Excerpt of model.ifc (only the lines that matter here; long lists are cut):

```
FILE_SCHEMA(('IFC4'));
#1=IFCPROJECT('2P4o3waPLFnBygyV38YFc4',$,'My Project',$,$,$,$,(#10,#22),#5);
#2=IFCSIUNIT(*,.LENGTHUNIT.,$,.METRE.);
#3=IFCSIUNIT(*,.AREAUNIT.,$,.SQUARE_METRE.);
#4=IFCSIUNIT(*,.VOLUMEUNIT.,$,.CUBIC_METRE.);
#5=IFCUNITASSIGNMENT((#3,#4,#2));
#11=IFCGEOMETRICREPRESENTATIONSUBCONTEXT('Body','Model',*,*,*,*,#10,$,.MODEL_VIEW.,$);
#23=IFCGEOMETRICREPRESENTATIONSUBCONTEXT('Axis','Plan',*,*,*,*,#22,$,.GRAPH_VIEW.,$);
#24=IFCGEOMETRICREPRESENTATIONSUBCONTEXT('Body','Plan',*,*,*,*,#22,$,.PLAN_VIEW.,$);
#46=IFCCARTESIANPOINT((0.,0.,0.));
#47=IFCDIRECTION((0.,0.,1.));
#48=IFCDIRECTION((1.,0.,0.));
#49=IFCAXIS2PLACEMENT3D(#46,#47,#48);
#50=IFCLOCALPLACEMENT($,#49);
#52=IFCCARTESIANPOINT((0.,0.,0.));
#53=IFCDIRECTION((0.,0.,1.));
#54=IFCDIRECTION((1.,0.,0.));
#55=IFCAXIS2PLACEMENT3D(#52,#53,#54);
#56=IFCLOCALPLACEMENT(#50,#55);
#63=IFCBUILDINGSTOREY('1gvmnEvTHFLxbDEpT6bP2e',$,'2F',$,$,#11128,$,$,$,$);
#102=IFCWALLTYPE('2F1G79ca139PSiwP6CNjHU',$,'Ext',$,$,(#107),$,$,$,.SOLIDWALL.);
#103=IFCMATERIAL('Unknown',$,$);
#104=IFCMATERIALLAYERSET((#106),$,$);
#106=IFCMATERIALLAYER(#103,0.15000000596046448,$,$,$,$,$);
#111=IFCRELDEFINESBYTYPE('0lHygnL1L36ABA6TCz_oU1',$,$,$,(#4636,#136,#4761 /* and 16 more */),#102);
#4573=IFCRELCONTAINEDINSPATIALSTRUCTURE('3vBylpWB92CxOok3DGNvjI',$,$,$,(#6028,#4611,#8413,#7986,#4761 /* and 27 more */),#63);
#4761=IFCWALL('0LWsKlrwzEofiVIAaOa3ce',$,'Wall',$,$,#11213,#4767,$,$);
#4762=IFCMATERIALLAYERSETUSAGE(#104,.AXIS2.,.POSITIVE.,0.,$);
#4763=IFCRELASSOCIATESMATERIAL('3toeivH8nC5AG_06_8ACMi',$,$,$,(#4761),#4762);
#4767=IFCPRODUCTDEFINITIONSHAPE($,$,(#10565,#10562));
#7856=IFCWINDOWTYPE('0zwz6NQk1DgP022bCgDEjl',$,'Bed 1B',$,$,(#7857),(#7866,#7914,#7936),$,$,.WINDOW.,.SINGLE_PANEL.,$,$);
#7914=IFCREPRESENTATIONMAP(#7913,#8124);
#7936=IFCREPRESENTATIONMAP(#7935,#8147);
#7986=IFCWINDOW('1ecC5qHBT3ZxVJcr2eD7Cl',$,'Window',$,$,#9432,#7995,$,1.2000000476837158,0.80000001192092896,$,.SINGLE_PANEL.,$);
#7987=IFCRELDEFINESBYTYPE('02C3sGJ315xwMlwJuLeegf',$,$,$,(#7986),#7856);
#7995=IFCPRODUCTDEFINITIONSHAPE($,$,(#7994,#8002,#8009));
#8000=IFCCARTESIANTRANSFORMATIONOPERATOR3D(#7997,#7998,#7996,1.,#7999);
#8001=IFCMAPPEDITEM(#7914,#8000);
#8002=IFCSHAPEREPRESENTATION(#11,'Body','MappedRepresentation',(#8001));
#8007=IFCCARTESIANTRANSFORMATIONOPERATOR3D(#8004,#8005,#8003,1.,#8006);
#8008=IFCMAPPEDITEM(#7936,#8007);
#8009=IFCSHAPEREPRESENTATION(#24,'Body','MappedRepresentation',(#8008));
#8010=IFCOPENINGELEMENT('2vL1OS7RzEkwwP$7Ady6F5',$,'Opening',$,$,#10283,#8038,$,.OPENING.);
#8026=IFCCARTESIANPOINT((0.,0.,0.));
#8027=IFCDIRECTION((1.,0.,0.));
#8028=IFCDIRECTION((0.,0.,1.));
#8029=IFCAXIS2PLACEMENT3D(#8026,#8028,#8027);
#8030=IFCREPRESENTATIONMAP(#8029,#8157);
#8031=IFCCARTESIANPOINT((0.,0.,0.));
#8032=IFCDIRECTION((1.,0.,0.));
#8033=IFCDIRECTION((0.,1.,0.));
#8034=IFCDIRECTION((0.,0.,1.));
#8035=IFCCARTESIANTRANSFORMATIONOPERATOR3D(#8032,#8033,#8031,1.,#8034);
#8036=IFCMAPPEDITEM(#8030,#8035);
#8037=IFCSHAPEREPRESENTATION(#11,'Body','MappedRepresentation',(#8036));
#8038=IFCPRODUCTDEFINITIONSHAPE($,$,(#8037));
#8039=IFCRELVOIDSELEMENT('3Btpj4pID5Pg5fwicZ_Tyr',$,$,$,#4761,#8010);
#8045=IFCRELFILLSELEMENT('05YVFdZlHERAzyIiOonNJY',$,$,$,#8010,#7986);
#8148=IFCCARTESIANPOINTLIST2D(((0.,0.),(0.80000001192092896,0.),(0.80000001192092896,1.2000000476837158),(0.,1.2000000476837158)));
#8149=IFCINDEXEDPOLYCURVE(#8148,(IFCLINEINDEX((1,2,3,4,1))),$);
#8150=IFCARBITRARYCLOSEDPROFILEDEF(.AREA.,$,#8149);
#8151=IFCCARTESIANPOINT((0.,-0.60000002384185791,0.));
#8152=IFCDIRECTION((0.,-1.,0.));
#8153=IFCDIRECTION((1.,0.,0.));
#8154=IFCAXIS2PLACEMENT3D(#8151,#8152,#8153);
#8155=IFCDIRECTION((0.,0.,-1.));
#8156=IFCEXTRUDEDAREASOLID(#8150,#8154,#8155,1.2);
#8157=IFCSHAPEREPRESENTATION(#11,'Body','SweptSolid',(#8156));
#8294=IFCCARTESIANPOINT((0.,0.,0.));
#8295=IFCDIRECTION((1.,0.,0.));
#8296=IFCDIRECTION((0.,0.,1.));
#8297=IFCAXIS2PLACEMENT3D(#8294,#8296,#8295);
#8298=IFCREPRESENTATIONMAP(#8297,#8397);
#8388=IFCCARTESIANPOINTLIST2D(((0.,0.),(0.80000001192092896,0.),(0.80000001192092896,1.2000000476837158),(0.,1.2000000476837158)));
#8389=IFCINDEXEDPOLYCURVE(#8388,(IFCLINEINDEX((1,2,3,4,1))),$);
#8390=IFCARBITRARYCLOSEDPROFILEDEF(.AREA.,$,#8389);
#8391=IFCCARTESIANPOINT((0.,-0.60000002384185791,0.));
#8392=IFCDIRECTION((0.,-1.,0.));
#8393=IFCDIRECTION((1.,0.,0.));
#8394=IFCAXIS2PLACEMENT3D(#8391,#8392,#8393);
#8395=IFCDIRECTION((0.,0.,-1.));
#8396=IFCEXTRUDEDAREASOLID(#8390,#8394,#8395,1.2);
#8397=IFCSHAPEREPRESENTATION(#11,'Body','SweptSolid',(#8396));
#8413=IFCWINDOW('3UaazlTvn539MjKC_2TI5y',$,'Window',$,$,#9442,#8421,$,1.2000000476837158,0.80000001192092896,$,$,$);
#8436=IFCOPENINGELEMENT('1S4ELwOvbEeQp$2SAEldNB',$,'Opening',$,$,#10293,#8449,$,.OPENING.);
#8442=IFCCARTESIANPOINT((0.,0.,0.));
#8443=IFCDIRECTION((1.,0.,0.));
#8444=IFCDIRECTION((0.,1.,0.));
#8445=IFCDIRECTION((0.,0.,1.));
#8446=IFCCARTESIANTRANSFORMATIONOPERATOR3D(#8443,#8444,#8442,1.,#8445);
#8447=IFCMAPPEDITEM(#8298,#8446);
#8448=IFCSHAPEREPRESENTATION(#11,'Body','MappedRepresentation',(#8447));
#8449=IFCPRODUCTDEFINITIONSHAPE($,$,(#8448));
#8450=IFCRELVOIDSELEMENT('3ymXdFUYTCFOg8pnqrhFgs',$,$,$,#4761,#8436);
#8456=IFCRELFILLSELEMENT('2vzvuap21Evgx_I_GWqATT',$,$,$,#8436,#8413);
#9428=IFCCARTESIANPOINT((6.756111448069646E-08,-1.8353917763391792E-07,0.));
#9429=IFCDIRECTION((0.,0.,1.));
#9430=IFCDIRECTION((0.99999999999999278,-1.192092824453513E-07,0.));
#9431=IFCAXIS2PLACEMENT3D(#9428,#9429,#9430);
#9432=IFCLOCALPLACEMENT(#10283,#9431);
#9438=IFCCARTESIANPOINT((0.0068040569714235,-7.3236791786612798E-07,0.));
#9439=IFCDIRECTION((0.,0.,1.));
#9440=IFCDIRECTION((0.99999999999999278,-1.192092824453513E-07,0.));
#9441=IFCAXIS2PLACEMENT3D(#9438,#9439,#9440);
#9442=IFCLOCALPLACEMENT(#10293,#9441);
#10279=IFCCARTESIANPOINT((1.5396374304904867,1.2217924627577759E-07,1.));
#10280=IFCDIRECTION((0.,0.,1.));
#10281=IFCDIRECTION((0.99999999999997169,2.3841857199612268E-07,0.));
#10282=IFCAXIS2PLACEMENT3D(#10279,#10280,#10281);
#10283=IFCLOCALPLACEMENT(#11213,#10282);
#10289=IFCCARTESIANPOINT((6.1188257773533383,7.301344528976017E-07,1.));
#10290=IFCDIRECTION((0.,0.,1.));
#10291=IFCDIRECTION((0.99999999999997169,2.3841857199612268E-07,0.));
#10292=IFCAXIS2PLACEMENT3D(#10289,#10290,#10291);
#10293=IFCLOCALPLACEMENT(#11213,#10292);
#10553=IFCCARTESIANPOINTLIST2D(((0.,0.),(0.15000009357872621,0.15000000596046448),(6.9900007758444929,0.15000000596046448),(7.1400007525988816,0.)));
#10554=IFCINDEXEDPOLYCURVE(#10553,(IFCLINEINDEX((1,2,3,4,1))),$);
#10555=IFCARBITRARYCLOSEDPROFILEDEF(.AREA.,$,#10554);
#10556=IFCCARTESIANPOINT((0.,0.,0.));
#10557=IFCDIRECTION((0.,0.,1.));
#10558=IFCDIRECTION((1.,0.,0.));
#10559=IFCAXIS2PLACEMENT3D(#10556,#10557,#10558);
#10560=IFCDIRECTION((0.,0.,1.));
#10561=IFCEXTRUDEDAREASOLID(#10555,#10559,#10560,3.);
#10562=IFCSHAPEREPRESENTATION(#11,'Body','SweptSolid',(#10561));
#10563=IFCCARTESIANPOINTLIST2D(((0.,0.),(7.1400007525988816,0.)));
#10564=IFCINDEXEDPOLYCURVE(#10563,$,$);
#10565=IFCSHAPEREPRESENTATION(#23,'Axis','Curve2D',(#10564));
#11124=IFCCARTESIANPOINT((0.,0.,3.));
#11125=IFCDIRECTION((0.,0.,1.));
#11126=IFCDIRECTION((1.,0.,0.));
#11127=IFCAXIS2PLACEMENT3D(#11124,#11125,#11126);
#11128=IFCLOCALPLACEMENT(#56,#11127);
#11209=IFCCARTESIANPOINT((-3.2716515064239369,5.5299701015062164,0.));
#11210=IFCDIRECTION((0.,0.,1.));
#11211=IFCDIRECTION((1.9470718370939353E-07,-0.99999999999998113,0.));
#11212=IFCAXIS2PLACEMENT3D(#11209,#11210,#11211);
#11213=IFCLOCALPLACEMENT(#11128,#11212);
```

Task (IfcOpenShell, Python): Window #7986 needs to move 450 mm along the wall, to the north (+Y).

```python
import ifcopenshell
import ifcopenshell.api.geometry
import ifcopenshell.util.placement

model = ifcopenshell.open("model.ifc")

window = model.by_guid("1ecC5qHBT3ZxVJcr2eD7Cl")
opening = window.FillsVoids[0].RelatingOpeningElement
wall = opening.VoidsElements[0].RelatingBuildingElement

wall_matrix = ifcopenshell.util.placement.get_local_placement(wall.ObjectPlacement)
shift = wall_matrix[:3, 0] * -0.45
before = ifcopenshell.util.placement.get_local_placement(window.ObjectPlacement)[:3, 3].copy()

# The window is placed relative to its opening, so it follows when the opening moves.
matrix = ifcopenshell.util.placement.get_local_placement(opening.ObjectPlacement)
matrix[:3, 3] += shift
ifcopenshell.api.geometry.edit_object_placement(
    model, product=opening, matrix=matrix, is_si=False, should_transform_children=True
)

after = ifcopenshell.util.placement.get_local_placement(window.ObjectPlacement)[:3, 3]
print("window moved by", (after - before).round(3) + 0.0)

model.write("model_updated.ifc")
```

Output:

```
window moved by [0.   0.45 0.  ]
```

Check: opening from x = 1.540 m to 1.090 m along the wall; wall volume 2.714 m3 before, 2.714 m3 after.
